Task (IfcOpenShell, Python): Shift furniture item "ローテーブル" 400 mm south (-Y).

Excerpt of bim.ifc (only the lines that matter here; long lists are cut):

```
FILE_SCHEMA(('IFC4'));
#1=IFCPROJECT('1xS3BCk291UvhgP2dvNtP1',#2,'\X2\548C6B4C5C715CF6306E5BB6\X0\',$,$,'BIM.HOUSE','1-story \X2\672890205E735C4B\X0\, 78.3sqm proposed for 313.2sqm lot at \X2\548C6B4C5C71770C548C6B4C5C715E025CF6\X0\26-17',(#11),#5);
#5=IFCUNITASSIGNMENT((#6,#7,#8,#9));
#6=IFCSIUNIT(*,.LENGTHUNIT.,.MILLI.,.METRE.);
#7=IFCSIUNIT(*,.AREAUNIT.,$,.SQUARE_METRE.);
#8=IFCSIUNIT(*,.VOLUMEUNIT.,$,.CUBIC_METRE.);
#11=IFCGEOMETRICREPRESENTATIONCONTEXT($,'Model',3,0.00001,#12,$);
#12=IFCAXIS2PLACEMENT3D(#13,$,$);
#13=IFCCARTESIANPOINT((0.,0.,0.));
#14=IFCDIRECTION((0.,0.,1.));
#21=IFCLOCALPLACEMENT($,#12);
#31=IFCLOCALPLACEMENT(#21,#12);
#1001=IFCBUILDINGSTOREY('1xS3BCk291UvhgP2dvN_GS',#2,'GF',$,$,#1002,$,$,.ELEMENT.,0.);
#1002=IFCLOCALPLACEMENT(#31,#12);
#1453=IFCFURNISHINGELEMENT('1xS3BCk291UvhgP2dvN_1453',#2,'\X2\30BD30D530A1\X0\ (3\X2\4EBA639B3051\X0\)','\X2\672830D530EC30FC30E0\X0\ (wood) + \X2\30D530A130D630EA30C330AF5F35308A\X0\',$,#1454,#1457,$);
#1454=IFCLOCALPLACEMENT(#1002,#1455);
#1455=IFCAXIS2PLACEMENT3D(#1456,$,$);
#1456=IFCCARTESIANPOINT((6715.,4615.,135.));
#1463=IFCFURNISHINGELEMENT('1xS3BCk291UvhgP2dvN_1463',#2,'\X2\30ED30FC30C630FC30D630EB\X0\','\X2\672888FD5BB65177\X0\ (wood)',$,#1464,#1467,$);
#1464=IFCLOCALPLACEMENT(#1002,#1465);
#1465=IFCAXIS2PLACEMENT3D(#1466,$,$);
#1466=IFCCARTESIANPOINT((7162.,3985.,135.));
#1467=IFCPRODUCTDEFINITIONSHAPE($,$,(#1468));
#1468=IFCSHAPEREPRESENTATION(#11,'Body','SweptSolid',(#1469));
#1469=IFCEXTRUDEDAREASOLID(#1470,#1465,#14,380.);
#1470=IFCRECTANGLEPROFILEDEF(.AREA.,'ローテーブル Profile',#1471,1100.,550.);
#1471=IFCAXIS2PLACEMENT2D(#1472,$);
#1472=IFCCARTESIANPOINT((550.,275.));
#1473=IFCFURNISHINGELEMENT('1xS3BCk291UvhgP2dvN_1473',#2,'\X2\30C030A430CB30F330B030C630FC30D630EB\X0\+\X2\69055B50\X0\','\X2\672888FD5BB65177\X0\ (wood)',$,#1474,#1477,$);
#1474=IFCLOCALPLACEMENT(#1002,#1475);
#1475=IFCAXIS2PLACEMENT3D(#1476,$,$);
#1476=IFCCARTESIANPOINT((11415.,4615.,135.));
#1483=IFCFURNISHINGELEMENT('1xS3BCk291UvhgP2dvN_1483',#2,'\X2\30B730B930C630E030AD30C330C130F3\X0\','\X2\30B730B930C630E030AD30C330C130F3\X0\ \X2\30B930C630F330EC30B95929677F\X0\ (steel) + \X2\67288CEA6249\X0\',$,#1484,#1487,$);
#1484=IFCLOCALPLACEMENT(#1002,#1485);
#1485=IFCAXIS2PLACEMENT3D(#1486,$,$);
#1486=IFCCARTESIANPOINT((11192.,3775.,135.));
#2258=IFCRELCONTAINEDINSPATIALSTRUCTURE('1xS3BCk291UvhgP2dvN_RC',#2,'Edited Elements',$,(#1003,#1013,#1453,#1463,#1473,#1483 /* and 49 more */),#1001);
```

```python
import ifcopenshell
import ifcopenshell.api.geometry
import ifcopenshell.util.placement

model = ifcopenshell.open("bim.ifc")

item = model.by_guid("1xS3BCk291UvhgP2dvN_1463")
matrix = ifcopenshell.util.placement.get_local_placement(item.ObjectPlacement)
matrix[1, 3] -= 400.0
ifcopenshell.api.geometry.edit_object_placement(model, product=item, matrix=matrix, is_si=False)

print(ifcopenshell.util.placement.get_local_placement(item.ObjectPlacement).round(3) + 0.0)

model.write("bim_updated.ifc")
```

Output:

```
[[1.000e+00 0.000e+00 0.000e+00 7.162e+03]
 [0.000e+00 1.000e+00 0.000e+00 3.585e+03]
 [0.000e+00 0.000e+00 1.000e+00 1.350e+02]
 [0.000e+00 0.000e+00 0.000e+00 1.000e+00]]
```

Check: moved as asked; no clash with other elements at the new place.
